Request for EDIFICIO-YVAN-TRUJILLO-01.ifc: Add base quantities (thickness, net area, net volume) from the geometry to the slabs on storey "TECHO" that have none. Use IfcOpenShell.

First a look at what the model holds.

```python
import ifcopenshell
import ifcopenshell.util.element
import ifcopenshell.util.unit

model = ifcopenshell.open("EDIFICIO-YVAN-TRUJILLO-01.ifc")
print(model.schema)
for unit_type in ("LENGTHUNIT", "AREAUNIT", "VOLUMEUNIT"):
    print(unit_type, ifcopenshell.util.unit.calculate_unit_scale(model, unit_type))
storey = next(s for s in model.by_type("IfcBuildingStorey") if s.Name == "TECHO")
slabs = [e for e in ifcopenshell.util.element.get_decomposition(storey) if e.is_a("IfcSlab")]
for e in sorted(slabs, key=lambda e: e.id()):
    print(e.id(), e.is_a(), e.Name, list(ifcopenshell.util.element.get_psets(e, qtos_only=True)), sep=" | ")
```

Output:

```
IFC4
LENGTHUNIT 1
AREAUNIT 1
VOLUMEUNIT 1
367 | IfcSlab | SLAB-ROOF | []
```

```python
import ifcopenshell
import ifcopenshell.api.pset
import ifcopenshell.geom
import ifcopenshell.util.element
import ifcopenshell.util.shape
import ifcopenshell.util.unit

model = ifcopenshell.open("EDIFICIO-YVAN-TRUJILLO-01.ifc")
unit_scale = ifcopenshell.util.unit.calculate_unit_scale(model)
area_scale = ifcopenshell.util.unit.calculate_unit_scale(model, "AREAUNIT")
volume_scale = ifcopenshell.util.unit.calculate_unit_scale(model, "VOLUMEUNIT")
settings = ifcopenshell.geom.settings()

storey = next(s for s in model.by_type("IfcBuildingStorey") if s.Name == "TECHO")
slabs = [e for e in ifcopenshell.util.element.get_decomposition(storey) if e.is_a("IfcSlab")]

for e in sorted(slabs, key=lambda e: e.id()):
    if ifcopenshell.util.element.get_psets(e, qtos_only=True, should_inherit=False):
        continue
    # Geometry comes back in metres, in the element's own axes.
    shape = ifcopenshell.geom.create_shape(settings, e)
    values = {
        "Width": ifcopenshell.util.shape.get_z(shape.geometry) / unit_scale,
        "NetArea": ifcopenshell.util.shape.get_footprint_area(shape.geometry) / area_scale,
        "NetVolume": ifcopenshell.util.shape.get_volume(shape.geometry) / volume_scale,
    }
    qto = ifcopenshell.api.pset.add_qto(model, product=e, name="Qto_SlabBaseQuantities")
    ifcopenshell.api.pset.edit_qto(model, qto=qto, properties=values)
    print(e.id(), {k: round(v, 3) for k, v in values.items()})

model.write("EDIFICIO-YVAN-TRUJILLO-01_rev.ifc")
```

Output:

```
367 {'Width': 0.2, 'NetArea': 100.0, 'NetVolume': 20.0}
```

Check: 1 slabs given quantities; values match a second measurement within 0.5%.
